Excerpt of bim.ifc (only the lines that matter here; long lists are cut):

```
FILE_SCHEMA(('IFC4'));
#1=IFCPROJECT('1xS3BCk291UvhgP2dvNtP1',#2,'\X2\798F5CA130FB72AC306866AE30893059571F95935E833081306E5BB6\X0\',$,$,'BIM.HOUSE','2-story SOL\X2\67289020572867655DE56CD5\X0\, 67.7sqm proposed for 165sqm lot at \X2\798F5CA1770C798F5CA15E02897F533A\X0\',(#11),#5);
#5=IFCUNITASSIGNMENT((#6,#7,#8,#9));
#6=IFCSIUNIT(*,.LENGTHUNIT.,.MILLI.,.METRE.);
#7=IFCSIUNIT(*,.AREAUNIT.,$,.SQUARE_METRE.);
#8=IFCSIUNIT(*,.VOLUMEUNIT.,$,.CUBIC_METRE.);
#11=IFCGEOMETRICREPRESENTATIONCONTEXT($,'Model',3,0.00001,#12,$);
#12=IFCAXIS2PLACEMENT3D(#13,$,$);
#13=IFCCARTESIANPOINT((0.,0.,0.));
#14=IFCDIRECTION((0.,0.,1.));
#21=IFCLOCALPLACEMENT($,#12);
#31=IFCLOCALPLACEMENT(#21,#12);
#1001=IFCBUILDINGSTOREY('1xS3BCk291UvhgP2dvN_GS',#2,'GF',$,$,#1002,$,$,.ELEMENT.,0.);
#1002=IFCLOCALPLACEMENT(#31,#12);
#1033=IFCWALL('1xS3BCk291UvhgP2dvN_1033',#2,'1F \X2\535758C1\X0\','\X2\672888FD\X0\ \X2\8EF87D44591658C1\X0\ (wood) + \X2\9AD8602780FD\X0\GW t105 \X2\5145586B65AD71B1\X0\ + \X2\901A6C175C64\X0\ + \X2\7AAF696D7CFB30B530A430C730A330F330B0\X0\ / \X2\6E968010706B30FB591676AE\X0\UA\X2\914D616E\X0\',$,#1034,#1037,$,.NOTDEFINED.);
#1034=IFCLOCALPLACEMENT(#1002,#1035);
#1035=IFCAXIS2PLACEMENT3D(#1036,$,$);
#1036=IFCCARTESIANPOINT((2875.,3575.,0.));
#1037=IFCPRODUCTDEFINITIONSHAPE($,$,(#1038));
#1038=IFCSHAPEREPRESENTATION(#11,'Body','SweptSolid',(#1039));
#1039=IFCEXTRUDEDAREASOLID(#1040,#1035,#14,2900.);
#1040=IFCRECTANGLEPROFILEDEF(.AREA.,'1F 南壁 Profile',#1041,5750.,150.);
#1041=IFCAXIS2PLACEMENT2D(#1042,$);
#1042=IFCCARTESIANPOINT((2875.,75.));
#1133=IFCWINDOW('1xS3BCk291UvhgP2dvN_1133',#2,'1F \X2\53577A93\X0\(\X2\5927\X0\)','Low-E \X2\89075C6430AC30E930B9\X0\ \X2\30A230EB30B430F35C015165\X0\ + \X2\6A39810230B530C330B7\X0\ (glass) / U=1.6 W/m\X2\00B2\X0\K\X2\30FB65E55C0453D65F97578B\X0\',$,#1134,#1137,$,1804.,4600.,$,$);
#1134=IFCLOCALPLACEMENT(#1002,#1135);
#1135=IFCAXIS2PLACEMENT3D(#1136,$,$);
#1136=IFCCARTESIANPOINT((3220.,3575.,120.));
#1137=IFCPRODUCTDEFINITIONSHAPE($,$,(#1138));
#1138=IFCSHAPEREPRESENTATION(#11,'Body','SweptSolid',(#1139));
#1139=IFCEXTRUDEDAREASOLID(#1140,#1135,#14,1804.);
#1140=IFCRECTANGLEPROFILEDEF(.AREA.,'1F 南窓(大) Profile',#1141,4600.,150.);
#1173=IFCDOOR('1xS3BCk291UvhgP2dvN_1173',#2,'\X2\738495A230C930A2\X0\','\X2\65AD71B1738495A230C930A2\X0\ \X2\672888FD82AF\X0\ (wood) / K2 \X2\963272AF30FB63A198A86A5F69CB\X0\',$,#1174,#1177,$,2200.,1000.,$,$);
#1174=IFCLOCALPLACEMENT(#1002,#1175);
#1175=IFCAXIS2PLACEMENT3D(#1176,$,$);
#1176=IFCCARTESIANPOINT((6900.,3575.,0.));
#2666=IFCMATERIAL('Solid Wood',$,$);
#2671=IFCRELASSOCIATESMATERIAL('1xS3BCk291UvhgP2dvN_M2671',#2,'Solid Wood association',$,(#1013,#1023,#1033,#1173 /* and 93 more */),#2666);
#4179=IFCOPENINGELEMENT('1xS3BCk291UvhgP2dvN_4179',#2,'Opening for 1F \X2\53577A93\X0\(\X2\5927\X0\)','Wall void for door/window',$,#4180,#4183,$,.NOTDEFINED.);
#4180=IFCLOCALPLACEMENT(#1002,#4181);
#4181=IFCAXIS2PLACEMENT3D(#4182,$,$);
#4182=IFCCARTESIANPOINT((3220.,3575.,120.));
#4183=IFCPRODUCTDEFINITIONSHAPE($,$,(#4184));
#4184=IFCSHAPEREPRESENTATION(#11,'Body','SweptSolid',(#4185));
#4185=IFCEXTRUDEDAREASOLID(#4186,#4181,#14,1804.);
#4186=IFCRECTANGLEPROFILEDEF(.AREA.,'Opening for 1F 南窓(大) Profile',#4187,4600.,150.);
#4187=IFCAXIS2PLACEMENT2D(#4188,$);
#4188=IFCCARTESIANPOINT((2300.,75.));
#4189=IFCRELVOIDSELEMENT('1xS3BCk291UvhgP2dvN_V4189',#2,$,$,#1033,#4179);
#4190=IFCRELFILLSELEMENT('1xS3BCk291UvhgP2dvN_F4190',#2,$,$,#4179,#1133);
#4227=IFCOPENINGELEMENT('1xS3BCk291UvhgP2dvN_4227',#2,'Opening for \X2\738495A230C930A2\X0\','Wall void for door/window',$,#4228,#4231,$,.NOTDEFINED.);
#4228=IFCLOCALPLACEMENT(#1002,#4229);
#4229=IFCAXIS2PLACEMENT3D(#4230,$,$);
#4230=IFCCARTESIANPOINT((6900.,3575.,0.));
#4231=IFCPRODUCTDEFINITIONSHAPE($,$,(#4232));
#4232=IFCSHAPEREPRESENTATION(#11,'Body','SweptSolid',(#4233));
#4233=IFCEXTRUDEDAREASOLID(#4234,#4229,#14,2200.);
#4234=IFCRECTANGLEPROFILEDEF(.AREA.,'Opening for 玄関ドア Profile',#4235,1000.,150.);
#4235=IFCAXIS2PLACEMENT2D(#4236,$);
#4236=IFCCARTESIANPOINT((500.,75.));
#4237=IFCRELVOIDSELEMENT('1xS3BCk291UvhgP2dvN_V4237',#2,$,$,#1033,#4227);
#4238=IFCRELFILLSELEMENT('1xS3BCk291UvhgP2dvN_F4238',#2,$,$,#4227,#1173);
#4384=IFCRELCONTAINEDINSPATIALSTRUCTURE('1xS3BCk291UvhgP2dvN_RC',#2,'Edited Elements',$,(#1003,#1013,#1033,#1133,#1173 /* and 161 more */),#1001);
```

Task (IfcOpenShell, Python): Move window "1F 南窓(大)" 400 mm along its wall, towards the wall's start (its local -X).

```python
import ifcopenshell
import ifcopenshell.api.geometry
import ifcopenshell.util.placement

model = ifcopenshell.open("bim.ifc")

window = model.by_guid("1xS3BCk291UvhgP2dvN_1133")
opening = window.FillsVoids[0].RelatingOpeningElement
wall = opening.VoidsElements[0].RelatingBuildingElement

wall_matrix = ifcopenshell.util.placement.get_local_placement(wall.ObjectPlacement)
shift = wall_matrix[:3, 0] * -400.0
before = ifcopenshell.util.placement.get_local_placement(window.ObjectPlacement)[:3, 3].copy()

# The window is not placed relative to its opening, so move both.
for product in (opening, window):
    matrix = ifcopenshell.util.placement.get_local_placement(product.ObjectPlacement)
    matrix[:3, 3] += shift
    ifcopenshell.api.geometry.edit_object_placement(model, product=product, matrix=matrix, is_si=False)

after = ifcopenshell.util.placement.get_local_placement(window.ObjectPlacement)[:3, 3]
print("window moved by", (after - before).round(3) + 0.0)

model.write("bim_v2.ifc")
```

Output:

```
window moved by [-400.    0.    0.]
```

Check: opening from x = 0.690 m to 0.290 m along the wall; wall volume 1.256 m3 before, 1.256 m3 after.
